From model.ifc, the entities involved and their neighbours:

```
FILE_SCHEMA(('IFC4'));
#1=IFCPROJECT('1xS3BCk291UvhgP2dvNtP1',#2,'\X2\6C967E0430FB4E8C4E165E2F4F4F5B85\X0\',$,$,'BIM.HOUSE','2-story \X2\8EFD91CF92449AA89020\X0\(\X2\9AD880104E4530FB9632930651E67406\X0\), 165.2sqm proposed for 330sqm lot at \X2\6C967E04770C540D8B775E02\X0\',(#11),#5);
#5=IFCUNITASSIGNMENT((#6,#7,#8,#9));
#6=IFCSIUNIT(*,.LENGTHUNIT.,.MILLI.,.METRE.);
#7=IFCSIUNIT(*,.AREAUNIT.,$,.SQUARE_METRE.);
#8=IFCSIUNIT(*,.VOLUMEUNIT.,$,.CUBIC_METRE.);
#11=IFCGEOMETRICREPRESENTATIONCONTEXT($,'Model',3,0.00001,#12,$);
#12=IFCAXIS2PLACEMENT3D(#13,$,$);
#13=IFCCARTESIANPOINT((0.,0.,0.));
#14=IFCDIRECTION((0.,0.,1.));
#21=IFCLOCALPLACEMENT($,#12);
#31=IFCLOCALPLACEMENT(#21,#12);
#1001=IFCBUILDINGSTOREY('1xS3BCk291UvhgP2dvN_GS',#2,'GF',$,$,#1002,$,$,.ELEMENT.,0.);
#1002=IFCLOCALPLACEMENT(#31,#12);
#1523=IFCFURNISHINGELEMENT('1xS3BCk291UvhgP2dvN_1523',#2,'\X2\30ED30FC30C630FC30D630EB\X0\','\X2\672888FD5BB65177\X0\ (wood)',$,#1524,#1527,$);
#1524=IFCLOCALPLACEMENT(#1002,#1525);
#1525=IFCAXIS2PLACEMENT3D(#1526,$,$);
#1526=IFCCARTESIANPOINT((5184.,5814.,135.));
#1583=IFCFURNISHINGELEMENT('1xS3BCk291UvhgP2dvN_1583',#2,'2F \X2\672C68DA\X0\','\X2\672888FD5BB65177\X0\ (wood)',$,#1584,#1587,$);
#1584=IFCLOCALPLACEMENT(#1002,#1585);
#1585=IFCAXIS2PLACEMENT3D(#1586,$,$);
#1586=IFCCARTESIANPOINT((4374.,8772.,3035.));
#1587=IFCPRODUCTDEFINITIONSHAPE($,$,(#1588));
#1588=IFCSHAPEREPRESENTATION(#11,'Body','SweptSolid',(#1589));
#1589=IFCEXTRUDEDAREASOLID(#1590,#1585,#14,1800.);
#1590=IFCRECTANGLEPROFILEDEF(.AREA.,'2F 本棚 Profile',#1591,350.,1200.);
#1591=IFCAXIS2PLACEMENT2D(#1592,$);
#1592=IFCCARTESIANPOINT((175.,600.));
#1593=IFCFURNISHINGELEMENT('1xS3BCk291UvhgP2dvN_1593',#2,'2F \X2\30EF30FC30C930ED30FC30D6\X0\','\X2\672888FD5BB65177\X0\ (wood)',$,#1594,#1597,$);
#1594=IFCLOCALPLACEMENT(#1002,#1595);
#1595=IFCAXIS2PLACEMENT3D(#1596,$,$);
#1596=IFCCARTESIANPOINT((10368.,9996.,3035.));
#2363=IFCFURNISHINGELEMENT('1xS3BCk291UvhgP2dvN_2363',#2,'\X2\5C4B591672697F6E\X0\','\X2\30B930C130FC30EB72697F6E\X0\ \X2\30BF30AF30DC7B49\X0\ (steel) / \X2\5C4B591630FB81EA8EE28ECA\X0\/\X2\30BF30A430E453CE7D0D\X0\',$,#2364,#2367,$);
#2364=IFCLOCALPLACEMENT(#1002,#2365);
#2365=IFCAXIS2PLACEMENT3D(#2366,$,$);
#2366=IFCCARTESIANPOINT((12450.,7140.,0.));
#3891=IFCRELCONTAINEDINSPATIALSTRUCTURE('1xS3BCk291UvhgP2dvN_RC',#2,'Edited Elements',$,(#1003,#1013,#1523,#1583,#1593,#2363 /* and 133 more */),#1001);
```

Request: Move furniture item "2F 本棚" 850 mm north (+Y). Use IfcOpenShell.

```python
import ifcopenshell
import ifcopenshell.api.geometry
import ifcopenshell.util.placement
import ifcopenshell.util.unit

model = ifcopenshell.open("model.ifc")
unit_scale = ifcopenshell.util.unit.calculate_unit_scale(model)

item = model.by_id(1583)
matrix = ifcopenshell.util.placement.get_local_placement(item.ObjectPlacement)
matrix[1, 3] += 0.85 / unit_scale
ifcopenshell.api.geometry.edit_object_placement(model, product=item, matrix=matrix, is_si=False)

print(ifcopenshell.util.placement.get_local_placement(item.ObjectPlacement).round(3) + 0.0)

model.write("model_edited.ifc")
```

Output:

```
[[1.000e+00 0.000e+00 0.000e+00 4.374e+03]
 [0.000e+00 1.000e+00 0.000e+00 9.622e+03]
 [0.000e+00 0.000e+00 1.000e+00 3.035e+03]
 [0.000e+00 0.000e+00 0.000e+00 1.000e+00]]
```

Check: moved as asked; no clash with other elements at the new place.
